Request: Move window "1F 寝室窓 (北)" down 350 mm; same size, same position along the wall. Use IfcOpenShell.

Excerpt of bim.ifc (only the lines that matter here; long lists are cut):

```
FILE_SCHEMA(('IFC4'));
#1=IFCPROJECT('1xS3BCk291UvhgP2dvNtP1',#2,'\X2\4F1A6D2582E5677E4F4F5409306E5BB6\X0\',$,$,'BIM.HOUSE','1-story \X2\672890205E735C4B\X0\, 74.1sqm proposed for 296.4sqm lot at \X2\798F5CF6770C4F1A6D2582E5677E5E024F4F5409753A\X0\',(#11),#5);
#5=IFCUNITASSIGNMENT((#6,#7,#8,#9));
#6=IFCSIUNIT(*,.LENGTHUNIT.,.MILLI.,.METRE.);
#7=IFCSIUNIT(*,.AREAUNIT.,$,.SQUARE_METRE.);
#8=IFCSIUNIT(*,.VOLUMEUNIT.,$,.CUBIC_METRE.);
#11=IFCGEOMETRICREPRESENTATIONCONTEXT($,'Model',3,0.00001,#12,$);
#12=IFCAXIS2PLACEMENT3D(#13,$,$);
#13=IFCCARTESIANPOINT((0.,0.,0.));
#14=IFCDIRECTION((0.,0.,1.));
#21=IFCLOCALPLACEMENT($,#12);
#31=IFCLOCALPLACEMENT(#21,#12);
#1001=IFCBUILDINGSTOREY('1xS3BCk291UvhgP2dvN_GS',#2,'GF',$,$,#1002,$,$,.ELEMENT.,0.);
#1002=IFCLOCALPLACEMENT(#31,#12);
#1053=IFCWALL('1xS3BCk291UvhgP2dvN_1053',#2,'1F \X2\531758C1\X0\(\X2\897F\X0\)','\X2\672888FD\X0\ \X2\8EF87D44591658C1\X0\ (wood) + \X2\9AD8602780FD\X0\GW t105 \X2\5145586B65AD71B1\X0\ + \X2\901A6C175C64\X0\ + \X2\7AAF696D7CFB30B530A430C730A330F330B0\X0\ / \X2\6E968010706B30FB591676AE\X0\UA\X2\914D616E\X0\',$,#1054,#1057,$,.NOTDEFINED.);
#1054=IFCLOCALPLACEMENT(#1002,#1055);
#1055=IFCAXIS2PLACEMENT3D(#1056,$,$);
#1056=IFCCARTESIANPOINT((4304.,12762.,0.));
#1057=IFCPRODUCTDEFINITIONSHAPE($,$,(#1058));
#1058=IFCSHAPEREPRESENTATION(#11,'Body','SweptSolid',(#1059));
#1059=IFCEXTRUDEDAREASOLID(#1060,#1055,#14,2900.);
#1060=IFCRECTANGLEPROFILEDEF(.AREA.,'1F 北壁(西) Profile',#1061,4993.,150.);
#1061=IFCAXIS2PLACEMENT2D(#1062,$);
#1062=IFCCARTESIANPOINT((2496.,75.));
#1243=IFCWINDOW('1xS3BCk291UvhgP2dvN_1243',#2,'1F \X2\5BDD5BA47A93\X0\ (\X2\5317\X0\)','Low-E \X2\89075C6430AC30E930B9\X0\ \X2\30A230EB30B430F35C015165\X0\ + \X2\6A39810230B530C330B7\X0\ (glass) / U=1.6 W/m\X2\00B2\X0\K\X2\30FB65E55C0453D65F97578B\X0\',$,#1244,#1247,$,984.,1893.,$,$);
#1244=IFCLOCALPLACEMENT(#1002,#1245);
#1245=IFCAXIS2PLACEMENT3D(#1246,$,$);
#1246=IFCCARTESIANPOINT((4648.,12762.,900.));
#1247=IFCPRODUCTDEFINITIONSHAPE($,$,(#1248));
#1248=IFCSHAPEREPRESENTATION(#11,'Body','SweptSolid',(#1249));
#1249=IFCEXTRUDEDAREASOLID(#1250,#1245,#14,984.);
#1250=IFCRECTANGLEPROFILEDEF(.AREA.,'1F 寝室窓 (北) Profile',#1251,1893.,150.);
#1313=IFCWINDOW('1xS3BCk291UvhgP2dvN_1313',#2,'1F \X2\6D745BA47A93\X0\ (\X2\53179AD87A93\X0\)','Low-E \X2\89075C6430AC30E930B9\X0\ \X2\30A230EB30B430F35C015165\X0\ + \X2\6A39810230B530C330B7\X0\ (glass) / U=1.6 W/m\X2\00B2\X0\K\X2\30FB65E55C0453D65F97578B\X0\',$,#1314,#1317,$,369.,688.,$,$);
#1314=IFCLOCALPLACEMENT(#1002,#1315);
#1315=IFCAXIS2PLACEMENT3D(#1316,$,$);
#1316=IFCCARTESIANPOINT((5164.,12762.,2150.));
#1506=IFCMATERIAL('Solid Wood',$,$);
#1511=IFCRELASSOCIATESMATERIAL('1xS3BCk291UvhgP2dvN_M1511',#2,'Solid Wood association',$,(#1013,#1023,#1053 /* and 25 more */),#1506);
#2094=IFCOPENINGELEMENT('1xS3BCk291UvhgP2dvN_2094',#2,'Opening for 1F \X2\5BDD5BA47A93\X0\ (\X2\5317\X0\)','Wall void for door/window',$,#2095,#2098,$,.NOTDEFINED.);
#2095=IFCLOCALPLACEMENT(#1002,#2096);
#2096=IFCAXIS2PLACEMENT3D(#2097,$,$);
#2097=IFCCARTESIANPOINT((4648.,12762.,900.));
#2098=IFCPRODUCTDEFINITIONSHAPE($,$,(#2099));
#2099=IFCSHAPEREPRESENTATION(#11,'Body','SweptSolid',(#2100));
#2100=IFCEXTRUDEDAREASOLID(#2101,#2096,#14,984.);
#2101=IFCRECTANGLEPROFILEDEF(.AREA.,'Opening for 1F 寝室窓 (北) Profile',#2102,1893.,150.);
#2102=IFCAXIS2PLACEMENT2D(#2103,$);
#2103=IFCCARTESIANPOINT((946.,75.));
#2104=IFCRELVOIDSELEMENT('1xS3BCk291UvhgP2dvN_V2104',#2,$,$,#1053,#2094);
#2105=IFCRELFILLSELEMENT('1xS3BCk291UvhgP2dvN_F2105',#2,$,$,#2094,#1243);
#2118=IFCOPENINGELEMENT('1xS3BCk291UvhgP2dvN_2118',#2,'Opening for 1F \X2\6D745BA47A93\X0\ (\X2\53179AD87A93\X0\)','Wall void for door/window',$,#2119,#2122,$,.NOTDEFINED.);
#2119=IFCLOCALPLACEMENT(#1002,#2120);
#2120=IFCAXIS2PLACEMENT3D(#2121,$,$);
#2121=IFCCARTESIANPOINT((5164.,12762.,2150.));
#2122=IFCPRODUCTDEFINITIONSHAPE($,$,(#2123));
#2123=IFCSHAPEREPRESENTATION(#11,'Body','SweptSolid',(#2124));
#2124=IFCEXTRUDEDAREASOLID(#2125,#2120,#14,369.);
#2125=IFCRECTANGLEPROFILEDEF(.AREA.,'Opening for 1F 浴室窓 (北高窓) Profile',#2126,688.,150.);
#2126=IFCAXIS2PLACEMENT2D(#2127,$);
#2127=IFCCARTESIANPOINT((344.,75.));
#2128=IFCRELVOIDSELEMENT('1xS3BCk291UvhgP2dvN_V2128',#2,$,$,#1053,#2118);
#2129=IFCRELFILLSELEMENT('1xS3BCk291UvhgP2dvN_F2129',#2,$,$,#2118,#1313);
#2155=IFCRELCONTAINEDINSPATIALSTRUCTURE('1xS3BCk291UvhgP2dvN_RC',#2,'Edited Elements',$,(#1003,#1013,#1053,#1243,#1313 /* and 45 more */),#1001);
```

```python
import numpy as np
import ifcopenshell
import ifcopenshell.api.geometry
import ifcopenshell.util.placement
import ifcopenshell.util.unit

model = ifcopenshell.open("bim.ifc")
unit_scale = ifcopenshell.util.unit.calculate_unit_scale(model)

window = model.by_guid("1xS3BCk291UvhgP2dvN_1243")
opening = window.FillsVoids[0].RelatingOpeningElement
dz = -0.35 / unit_scale

shift = np.array([0.0, 0.0, dz])
# The window is not placed relative to its opening, so move both.
for product in (opening, window):
    matrix = ifcopenshell.util.placement.get_local_placement(product.ObjectPlacement)
    matrix[:3, 3] += shift
    ifcopenshell.api.geometry.edit_object_placement(model, product=product, matrix=matrix, is_si=False)

print(f"moved by {dz * unit_scale:+.3f} m")

model.write("bim_edited.ifc")
```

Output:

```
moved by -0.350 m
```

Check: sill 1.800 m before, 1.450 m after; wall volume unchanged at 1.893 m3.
